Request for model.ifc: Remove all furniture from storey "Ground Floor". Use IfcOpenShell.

First a look at what the model holds.

```python
import ifcopenshell
import ifcopenshell.util.element

model = ifcopenshell.open("model.ifc")
print(model.schema)
storey = next(s for s in model.by_type("IfcBuildingStorey") if s.Name == "Ground Floor")
furniture = [e for e in ifcopenshell.util.element.get_decomposition(storey) if e.is_a("IfcFurnishingElement")]
seen = {}
for e in furniture:
    element_type = ifcopenshell.util.element.get_type(e)
    name = element_type.Name if element_type not in (None, e) else None
    seen[name] = seen.get(name, 0) + 1
for name, count in sorted(seen.items(), key=str):
    print(count, "x", name)
```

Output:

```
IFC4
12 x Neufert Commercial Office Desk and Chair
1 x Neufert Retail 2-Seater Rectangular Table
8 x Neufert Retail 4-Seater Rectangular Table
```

```python
import ifcopenshell
import ifcopenshell.api.root
import ifcopenshell.util.element

model = ifcopenshell.open("model.ifc")

storey = next(s for s in model.by_type("IfcBuildingStorey") if s.Name == "Ground Floor")
furniture = [e for e in ifcopenshell.util.element.get_decomposition(storey) if e.is_a("IfcFurnishingElement")]

for e in furniture:
    ifcopenshell.api.root.remove_product(model, product=e)
print(len(furniture), "removed")

model.write("model_rev.ifc")
```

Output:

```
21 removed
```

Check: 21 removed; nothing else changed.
